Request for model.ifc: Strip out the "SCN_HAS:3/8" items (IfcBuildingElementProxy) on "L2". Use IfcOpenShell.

First a look at what the model holds.

```python
import ifcopenshell
import ifcopenshell.util.element

model = ifcopenshell.open("model.ifc")
print(model.schema)
storey = next(s for s in model.by_type("IfcBuildingStorey") if s.Name == "L2")
proxies = [e for e in ifcopenshell.util.element.get_decomposition(storey) if e.is_a("IfcBuildingElementProxy")]
seen = {}
for e in proxies:
    element_type = ifcopenshell.util.element.get_type(e)
    name = element_type.Name if element_type not in (None, e) else None
    seen[name] = seen.get(name, 0) + 1
for name, count in sorted(seen.items(), key=str):
    print(count, "x", name)
```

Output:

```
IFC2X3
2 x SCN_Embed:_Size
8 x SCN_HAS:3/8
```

```python
import ifcopenshell
import ifcopenshell.api.root
import ifcopenshell.util.element

model = ifcopenshell.open("model.ifc")

storey = next(s for s in model.by_type("IfcBuildingStorey") if s.Name == "L2")
proxies = [e for e in ifcopenshell.util.element.get_decomposition(storey) if e.is_a("IfcBuildingElementProxy")]
targets = [e for e in proxies if (t := ifcopenshell.util.element.get_type(e)) not in (None, e) and t.Name == "SCN_HAS:3/8"]

for e in targets:
    ifcopenshell.api.root.remove_product(model, product=e)
print(len(targets), "removed")

model.write("model-out.ifc")
```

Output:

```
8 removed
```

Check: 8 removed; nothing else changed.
